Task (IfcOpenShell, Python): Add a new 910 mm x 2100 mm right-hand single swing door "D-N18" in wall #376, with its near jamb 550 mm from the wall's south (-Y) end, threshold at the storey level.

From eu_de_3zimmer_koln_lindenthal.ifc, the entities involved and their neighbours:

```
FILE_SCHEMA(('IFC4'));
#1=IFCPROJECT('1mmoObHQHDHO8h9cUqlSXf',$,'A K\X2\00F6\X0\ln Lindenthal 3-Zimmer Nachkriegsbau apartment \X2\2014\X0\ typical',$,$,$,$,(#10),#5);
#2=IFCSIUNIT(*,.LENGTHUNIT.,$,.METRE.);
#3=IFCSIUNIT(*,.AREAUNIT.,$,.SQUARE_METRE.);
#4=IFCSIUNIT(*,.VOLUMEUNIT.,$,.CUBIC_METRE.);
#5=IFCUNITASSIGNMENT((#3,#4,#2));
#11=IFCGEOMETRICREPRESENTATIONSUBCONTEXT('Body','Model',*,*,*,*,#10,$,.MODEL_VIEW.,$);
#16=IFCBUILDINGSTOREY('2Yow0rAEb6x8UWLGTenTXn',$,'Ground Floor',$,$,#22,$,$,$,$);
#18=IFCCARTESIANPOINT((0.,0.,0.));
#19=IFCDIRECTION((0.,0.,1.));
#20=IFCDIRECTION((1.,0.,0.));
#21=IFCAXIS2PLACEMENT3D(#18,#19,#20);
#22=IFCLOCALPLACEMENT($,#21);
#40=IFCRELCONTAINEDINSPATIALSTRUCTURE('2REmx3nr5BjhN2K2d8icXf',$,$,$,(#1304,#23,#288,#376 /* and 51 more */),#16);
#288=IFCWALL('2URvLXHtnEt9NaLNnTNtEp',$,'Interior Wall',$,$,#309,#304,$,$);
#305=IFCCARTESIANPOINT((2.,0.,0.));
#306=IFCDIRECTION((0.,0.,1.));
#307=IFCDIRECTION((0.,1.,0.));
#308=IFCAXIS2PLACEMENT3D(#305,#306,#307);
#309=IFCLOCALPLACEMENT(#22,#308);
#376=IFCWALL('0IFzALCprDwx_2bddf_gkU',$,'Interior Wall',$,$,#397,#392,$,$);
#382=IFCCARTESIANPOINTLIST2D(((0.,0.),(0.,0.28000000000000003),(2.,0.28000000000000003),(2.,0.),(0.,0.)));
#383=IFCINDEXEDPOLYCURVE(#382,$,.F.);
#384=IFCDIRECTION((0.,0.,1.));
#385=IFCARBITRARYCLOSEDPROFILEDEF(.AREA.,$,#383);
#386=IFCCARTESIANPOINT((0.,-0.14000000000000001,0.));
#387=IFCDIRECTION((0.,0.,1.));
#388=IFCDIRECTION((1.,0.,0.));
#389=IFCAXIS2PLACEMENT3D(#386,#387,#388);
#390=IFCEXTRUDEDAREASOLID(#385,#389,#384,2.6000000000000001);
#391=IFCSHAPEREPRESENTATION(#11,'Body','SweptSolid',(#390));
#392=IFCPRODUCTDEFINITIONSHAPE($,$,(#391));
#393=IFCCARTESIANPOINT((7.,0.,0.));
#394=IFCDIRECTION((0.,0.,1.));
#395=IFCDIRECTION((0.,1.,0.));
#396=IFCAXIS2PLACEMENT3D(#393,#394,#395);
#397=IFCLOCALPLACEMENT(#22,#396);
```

```python
import numpy as np
import ifcopenshell
import ifcopenshell.api.feature
import ifcopenshell.api.geometry
import ifcopenshell.api.root
import ifcopenshell.api.spatial
import ifcopenshell.geom
import ifcopenshell.util.element
import ifcopenshell.util.placement
import ifcopenshell.util.representation
import ifcopenshell.util.shape
import ifcopenshell.util.unit

model = ifcopenshell.open("eu_de_3zimmer_koln_lindenthal.ifc")
unit_scale = ifcopenshell.util.unit.calculate_unit_scale(model)
settings = ifcopenshell.geom.settings()


def volume(element):
    """Net volume in cubic metres, openings subtracted."""
    shape = ifcopenshell.geom.create_shape(settings, element)
    return ifcopenshell.util.shape.get_volume(shape.geometry)


wall = model.by_id(376)
storey = ifcopenshell.util.element.get_container(wall, ifc_class="IfcBuildingStorey")
context = ifcopenshell.util.representation.get_context(model, "Model", "Body", "MODEL_VIEW")
before = volume(wall)

width, height, from_end, sill = 0.91, 2.1, 0.55, 0.0  # metres

# The wall runs along its own X axis, and the end named is its -X end.
wall_shape = ifcopenshell.geom.create_shape(settings, wall)
x, y, z = ifcopenshell.util.shape.get_vertices(wall_shape.geometry).T
start = x.min() + from_end
face, thickness = float(y.min()), float(y.max() - y.min())
wall_matrix = ifcopenshell.util.placement.get_local_placement(wall.ObjectPlacement)
level = ifcopenshell.util.placement.get_local_placement(storey.ObjectPlacement)[2, 3]


def in_wall(x, y):
    """Placement at x, y metres in the wall's axes, at sill height."""
    matrix = wall_matrix.copy()
    matrix[:, 3] = wall_matrix @ np.array([x / unit_scale, y / unit_scale, 0.0, 1.0])
    matrix[2, 3] = level + sill / unit_scale
    return matrix


# Opening: a box that overshoots both wall faces by 50 mm.
opening = ifcopenshell.api.root.create_entity(model, ifc_class="IfcOpeningElement", predefined_type="OPENING")
box = ifcopenshell.api.geometry.add_wall_representation(
    model, context=context, length=width, height=height, thickness=thickness + 0.1
)
ifcopenshell.api.geometry.assign_representation(model, product=opening, representation=box)
ifcopenshell.api.geometry.edit_object_placement(model, product=opening, matrix=in_wall(start, face - 0.05), is_si=False)
ifcopenshell.api.feature.add_feature(model, feature=opening, element=wall)

door = ifcopenshell.api.root.create_entity(model, ifc_class="IfcDoor", name="D-N18", predefined_type="DOOR")
door.OverallWidth, door.OverallHeight = width / unit_scale, height / unit_scale
door.OperationType = "SINGLE_SWING_RIGHT"
body = ifcopenshell.api.geometry.add_door_representation(
    model,
    context=context,
    overall_width=door.OverallWidth,
    overall_height=door.OverallHeight,
    operation_type="SINGLE_SWING_RIGHT",
    lining_properties={"LiningDepth": thickness / unit_scale, "ThresholdDepth": thickness / unit_scale},
)
ifcopenshell.api.geometry.assign_representation(model, product=door, representation=body)
ifcopenshell.api.spatial.assign_container(model, products=[door], relating_structure=storey)
ifcopenshell.api.feature.add_filling(model, opening=opening, element=door)

# The lining spans the wall, so the door starts at the wall face.
ifcopenshell.api.geometry.edit_object_placement(model, product=door, matrix=in_wall(start, face), is_si=False)

after = volume(wall)

print(f"wall volume {before:.3f} -> {after:.3f} m3")

model.write("eu_de_3zimmer_koln_lindenthal_rev.ifc")
```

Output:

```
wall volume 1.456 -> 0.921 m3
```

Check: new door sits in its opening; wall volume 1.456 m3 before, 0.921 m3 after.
